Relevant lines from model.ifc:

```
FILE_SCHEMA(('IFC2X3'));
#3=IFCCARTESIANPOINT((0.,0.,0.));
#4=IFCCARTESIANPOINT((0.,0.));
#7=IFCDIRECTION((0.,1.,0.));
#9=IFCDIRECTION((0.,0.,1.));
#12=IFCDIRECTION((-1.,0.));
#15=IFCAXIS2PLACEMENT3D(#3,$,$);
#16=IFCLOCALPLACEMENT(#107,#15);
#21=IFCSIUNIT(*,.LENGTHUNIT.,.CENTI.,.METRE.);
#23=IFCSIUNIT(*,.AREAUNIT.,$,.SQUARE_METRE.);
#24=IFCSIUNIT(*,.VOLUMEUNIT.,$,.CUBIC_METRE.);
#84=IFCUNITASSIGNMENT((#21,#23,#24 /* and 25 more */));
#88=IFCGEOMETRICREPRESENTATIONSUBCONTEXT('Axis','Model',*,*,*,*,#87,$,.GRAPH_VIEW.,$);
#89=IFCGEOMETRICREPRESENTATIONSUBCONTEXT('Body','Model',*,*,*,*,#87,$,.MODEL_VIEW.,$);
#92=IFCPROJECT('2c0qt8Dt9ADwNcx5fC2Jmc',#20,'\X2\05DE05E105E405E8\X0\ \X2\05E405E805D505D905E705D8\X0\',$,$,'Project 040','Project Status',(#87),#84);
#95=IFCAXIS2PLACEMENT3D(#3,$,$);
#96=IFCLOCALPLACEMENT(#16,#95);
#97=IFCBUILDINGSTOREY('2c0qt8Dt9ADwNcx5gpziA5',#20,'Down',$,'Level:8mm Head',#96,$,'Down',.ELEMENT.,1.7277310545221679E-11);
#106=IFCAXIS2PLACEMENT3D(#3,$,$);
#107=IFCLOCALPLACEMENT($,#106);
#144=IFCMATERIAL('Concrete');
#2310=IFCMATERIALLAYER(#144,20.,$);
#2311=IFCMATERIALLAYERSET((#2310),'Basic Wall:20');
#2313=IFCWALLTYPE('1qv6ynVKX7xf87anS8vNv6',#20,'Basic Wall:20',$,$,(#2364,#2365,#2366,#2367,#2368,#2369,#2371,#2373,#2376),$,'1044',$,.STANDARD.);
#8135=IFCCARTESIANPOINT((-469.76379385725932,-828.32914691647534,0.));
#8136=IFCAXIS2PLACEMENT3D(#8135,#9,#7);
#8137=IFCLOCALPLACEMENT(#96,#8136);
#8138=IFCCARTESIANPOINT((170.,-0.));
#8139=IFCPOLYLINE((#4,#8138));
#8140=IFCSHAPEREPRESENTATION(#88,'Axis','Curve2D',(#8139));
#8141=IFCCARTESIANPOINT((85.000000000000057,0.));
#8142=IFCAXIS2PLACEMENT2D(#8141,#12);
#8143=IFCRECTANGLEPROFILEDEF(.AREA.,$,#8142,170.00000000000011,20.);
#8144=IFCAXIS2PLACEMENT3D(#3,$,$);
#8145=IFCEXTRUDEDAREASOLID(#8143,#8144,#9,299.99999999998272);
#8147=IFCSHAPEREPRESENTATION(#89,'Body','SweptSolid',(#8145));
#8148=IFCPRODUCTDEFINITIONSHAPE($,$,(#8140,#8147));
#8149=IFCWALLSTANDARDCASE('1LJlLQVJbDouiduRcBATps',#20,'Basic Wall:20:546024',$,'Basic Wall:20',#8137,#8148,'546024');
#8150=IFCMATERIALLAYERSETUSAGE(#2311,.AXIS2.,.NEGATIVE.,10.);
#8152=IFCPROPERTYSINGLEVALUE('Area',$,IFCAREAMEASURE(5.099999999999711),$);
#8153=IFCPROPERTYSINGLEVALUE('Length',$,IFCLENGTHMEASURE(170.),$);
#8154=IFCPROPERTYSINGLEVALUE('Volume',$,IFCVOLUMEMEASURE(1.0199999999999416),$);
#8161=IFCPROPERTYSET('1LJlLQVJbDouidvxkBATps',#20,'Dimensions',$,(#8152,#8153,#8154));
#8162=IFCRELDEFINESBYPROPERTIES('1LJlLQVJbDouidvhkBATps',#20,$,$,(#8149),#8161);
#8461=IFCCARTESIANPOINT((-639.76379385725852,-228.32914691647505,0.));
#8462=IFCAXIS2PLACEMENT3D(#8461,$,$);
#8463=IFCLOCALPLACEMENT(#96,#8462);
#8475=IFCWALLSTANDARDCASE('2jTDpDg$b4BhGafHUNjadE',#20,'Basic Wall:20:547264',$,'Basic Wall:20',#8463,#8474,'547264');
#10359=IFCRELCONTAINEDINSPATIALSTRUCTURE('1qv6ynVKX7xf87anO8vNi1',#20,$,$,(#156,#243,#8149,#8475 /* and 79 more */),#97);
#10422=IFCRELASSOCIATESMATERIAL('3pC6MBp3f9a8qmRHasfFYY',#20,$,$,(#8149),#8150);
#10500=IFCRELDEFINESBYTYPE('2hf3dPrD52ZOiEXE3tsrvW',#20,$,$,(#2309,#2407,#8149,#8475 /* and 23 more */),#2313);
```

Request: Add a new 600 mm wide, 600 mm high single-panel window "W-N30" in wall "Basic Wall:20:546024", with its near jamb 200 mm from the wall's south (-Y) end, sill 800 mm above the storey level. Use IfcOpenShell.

```python
import numpy as np
import ifcopenshell
import ifcopenshell.api.feature
import ifcopenshell.api.geometry
import ifcopenshell.api.pset
import ifcopenshell.api.root
import ifcopenshell.api.spatial
import ifcopenshell.api.type
import ifcopenshell.geom
import ifcopenshell.util.element
import ifcopenshell.util.placement
import ifcopenshell.util.representation
import ifcopenshell.util.shape
import ifcopenshell.util.unit

model = ifcopenshell.open("model.ifc")
unit_scale = ifcopenshell.util.unit.calculate_unit_scale(model)
area_scale = ifcopenshell.util.unit.calculate_unit_scale(model, "AREAUNIT")
volume_scale = ifcopenshell.util.unit.calculate_unit_scale(model, "VOLUMEUNIT")
settings = ifcopenshell.geom.settings()


def volume(element):
    """Net volume in cubic metres, openings subtracted."""
    shape = ifcopenshell.geom.create_shape(settings, element)
    return ifcopenshell.util.shape.get_volume(shape.geometry)


wall = model.by_id(8149)
storey = ifcopenshell.util.element.get_container(wall, ifc_class="IfcBuildingStorey")
context = ifcopenshell.util.representation.get_context(model, "Model", "Body", "MODEL_VIEW")
before = volume(wall)

width, height, from_end, sill = 0.6, 0.6, 0.2, 0.8  # metres

# The wall runs along its own X axis, and the end named is its -X end.
wall_shape = ifcopenshell.geom.create_shape(settings, wall)
x, y, z = ifcopenshell.util.shape.get_vertices(wall_shape.geometry).T
start = x.min() + from_end
face, thickness = float(y.min()), float(y.max() - y.min())
wall_matrix = ifcopenshell.util.placement.get_local_placement(wall.ObjectPlacement)
level = ifcopenshell.util.placement.get_local_placement(storey.ObjectPlacement)[2, 3]


def in_wall(x, y):
    """Placement at x, y metres in the wall's axes, at sill height."""
    matrix = wall_matrix.copy()
    matrix[:, 3] = wall_matrix @ np.array([x / unit_scale, y / unit_scale, 0.0, 1.0])
    matrix[2, 3] = level + sill / unit_scale
    return matrix


# Opening: a box that overshoots both wall faces by 50 mm.
opening = ifcopenshell.api.root.create_entity(model, ifc_class="IfcOpeningElement")
box = ifcopenshell.api.geometry.add_wall_representation(
    model, context=context, length=width, height=height, thickness=thickness + 0.1
)
ifcopenshell.api.geometry.assign_representation(model, product=opening, representation=box)
ifcopenshell.api.geometry.edit_object_placement(model, product=opening, matrix=in_wall(start, face - 0.05), is_si=False)
ifcopenshell.api.feature.add_feature(model, feature=opening, element=wall)

window = ifcopenshell.api.root.create_entity(model, ifc_class="IfcWindow", name="W-N30")
window.OverallWidth, window.OverallHeight = width / unit_scale, height / unit_scale
body = ifcopenshell.api.geometry.add_window_representation(
    model,
    context=context,
    overall_width=window.OverallWidth,
    overall_height=window.OverallHeight,
    partition_type="SINGLE_PANEL",
)
ifcopenshell.api.geometry.assign_representation(model, product=window, representation=body)
ifcopenshell.api.spatial.assign_container(model, products=[window], relating_structure=storey)
fills = ifcopenshell.api.feature.add_filling(model, opening=opening, element=window)
fills.OwnerHistory = window.OwnerHistory  # required in IFC2X3

# IFC2X3 keeps the operation on the window style.
style = ifcopenshell.api.root.create_entity(model, ifc_class="IfcWindowStyle", name="W-N30")
style.OperationType, style.ConstructionType = "SINGLE_PANEL", "NOTDEFINED"
style.ParameterTakesPrecedence = style.Sizeable = False
ifcopenshell.api.type.assign_type(model, related_objects=[window], relating_type=style)

# Centre the window in the wall's thickness.
ifcopenshell.api.geometry.edit_object_placement(model, product=window, matrix=in_wall(start, face), is_si=False)
window_shape = ifcopenshell.geom.create_shape(settings, window)
depth = ifcopenshell.util.shape.get_vertices(window_shape.geometry)[:, 1]
offset = face + thickness / 2 - (depth.min() + depth.max()) / 2
ifcopenshell.api.geometry.edit_object_placement(model, product=window, matrix=in_wall(start, offset), is_si=False)

after = volume(wall)

# Update the wall's stored quantities.
pset = model.by_id(ifcopenshell.util.element.get_pset(wall, "Dimensions", should_inherit=False)["id"])
ifcopenshell.api.pset.edit_pset(model, pset=pset, properties={
    "Area": model.create_entity("IfcAreaMeasure", after / thickness / area_scale),
    "Volume": model.create_entity("IfcVolumeMeasure", after / volume_scale),
})

print(f"wall volume {before:.3f} -> {after:.3f} m3")

model.write("model_edited.ifc")
```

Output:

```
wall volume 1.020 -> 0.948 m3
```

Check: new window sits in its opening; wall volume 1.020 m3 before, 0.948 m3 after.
